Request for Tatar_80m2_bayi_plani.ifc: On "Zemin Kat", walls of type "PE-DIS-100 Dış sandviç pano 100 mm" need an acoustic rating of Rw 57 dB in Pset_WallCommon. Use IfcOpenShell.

First a look at what the model holds.

```python
import ifcopenshell
import ifcopenshell.util.element

model = ifcopenshell.open("Tatar_80m2_bayi_plani.ifc")
print(model.schema)
storey = next(s for s in model.by_type("IfcBuildingStorey") if s.Name == "Zemin Kat")
walls = [e for e in ifcopenshell.util.element.get_decomposition(storey) if e.is_a("IfcWall")]
seen = {}
for e in walls:
    element_type = ifcopenshell.util.element.get_type(e)
    key = (element_type.Name if element_type != e and element_type else None, ifcopenshell.util.element.get_pset(e, "Pset_WallCommon", "AcousticRating"))
    seen[key] = seen.get(key, 0) + 1
for (name, value), count in sorted(seen.items(), key=str):
    print(count, "x", name, "|", value)
```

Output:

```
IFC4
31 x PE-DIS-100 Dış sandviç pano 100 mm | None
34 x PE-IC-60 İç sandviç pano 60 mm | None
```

```python
import ifcopenshell
import ifcopenshell.api.pset
import ifcopenshell.util.element

model = ifcopenshell.open("Tatar_80m2_bayi_plani.ifc")

storey = next(s for s in model.by_type("IfcBuildingStorey") if s.Name == "Zemin Kat")
walls = [e for e in ifcopenshell.util.element.get_decomposition(storey) if e.is_a("IfcWall")]

count = 0
for e in walls:
    element_type = ifcopenshell.util.element.get_type(e)
    if element_type in (None, e) or element_type.Name != "PE-DIS-100 Dış sandviç pano 100 mm":
        continue
    # add_pset returns the element's existing set when there is one.
    pset = ifcopenshell.api.pset.add_pset(model, product=e, name="Pset_WallCommon")
    ifcopenshell.api.pset.edit_pset(model, pset=pset, properties={"AcousticRating": "Rw 57 dB"})
    count += 1

print(count, "walls updated")

model.write("Tatar_80m2_bayi_plani_v2.ifc")
```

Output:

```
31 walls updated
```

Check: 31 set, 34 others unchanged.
